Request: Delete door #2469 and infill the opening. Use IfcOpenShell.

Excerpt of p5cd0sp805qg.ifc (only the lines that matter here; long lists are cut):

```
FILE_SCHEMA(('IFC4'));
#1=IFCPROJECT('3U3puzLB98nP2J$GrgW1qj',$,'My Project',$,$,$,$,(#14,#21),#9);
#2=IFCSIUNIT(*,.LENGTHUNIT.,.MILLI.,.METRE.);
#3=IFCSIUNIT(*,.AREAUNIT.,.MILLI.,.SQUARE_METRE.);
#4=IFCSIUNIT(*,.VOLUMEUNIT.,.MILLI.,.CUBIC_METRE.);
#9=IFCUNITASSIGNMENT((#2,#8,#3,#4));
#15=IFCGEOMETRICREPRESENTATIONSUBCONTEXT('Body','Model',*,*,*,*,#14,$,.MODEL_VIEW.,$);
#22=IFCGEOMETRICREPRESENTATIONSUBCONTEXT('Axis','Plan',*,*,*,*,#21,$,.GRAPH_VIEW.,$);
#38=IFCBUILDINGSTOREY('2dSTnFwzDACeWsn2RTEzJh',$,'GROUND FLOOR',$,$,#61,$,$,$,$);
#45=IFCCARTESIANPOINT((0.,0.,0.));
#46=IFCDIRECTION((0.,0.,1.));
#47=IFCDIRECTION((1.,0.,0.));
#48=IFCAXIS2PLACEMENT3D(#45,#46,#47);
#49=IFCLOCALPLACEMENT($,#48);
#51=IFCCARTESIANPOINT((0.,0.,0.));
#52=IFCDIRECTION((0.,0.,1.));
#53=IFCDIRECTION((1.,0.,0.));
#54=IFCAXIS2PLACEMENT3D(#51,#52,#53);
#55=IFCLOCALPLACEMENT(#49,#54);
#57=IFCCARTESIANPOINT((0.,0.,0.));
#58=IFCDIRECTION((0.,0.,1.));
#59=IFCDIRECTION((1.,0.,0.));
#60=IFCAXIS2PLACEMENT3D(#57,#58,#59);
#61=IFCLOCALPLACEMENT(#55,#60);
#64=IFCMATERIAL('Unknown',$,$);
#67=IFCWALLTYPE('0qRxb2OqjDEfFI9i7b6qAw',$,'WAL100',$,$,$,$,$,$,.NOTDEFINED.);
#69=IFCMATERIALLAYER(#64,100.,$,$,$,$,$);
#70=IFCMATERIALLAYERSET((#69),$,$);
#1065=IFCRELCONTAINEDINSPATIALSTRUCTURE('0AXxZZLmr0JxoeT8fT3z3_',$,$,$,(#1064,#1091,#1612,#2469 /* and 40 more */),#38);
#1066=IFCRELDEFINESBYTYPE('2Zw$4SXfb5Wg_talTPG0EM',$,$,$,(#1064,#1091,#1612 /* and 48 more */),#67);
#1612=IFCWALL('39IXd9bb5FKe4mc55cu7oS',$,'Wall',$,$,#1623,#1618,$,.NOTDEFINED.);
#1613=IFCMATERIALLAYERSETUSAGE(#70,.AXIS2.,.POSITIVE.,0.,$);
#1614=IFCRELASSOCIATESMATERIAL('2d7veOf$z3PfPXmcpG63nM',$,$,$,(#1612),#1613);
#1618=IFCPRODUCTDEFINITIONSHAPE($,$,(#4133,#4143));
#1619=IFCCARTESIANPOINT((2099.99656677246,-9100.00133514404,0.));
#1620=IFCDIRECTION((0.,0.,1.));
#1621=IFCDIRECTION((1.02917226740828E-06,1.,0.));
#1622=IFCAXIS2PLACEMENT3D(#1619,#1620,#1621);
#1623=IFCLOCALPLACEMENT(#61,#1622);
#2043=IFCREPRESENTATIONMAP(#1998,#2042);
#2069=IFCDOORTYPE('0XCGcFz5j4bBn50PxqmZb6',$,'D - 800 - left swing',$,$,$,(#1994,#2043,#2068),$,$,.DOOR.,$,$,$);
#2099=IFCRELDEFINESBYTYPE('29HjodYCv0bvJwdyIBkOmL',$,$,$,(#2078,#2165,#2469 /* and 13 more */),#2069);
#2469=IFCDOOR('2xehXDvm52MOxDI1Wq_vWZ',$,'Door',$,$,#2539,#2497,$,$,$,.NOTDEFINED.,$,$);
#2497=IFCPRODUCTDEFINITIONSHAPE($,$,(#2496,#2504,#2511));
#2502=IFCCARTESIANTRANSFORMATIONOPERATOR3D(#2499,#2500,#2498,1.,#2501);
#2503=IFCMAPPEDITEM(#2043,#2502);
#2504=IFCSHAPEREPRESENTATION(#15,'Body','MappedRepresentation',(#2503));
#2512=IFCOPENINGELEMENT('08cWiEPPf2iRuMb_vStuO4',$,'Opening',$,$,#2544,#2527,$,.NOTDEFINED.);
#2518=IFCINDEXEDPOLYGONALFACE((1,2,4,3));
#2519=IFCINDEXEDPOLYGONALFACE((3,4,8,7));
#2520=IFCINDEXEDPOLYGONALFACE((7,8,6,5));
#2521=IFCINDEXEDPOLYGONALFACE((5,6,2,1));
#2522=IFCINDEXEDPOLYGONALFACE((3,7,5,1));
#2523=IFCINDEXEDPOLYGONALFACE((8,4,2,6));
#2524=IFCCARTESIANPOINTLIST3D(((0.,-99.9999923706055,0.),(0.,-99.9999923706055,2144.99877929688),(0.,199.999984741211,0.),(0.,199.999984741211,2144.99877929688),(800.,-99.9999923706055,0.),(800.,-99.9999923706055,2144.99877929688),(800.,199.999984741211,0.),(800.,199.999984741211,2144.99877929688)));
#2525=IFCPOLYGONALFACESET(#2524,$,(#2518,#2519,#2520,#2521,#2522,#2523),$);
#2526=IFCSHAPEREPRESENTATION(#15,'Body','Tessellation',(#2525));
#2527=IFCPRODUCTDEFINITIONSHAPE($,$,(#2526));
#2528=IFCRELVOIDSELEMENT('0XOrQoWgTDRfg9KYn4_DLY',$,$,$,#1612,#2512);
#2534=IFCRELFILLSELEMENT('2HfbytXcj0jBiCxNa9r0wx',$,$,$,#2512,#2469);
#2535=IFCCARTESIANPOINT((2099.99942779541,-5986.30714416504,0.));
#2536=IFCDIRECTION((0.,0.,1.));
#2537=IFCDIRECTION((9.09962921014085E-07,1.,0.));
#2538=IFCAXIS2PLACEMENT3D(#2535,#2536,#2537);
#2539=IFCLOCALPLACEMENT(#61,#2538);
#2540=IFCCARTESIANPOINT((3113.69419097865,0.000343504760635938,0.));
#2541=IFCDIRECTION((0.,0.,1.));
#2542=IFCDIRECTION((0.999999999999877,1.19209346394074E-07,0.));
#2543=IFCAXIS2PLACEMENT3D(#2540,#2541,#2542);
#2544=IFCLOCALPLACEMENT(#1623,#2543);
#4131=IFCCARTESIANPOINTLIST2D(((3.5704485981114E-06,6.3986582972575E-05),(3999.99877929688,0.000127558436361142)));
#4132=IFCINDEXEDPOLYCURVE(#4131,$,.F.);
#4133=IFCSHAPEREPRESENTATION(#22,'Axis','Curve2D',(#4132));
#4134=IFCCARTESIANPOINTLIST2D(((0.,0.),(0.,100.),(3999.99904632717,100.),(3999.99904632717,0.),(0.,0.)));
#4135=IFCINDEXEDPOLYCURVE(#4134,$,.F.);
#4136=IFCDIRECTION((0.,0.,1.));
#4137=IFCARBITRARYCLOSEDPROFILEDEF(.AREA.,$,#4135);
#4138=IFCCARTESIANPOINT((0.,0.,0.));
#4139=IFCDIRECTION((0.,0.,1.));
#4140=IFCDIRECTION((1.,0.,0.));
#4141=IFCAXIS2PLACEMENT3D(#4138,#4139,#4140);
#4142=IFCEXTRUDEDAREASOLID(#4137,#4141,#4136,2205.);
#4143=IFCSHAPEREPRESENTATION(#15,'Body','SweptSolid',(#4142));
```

```python
import ifcopenshell
import ifcopenshell.api.feature
import ifcopenshell.api.root
import ifcopenshell.geom
import ifcopenshell.util.shape

model = ifcopenshell.open("p5cd0sp805qg.ifc")
settings = ifcopenshell.geom.settings()


def volume(element):
    """Net volume in cubic metres, openings subtracted."""
    shape = ifcopenshell.geom.create_shape(settings, element)
    return ifcopenshell.util.shape.get_volume(shape.geometry)


door = model.by_guid("2xehXDvm52MOxDI1Wq_vWZ")
opening = door.FillsVoids[0].RelatingOpeningElement
wall = opening.VoidsElements[0].RelatingBuildingElement
before = volume(wall)

ifcopenshell.api.root.remove_product(model, product=door)
ifcopenshell.api.feature.remove_feature(model, feature=opening)

after = volume(wall)

print(f"wall volume {before:.3f} -> {after:.3f} m3")

model.write("p5cd0sp805qg_updated.ifc")
```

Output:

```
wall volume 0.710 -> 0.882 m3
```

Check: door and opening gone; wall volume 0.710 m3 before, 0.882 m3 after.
